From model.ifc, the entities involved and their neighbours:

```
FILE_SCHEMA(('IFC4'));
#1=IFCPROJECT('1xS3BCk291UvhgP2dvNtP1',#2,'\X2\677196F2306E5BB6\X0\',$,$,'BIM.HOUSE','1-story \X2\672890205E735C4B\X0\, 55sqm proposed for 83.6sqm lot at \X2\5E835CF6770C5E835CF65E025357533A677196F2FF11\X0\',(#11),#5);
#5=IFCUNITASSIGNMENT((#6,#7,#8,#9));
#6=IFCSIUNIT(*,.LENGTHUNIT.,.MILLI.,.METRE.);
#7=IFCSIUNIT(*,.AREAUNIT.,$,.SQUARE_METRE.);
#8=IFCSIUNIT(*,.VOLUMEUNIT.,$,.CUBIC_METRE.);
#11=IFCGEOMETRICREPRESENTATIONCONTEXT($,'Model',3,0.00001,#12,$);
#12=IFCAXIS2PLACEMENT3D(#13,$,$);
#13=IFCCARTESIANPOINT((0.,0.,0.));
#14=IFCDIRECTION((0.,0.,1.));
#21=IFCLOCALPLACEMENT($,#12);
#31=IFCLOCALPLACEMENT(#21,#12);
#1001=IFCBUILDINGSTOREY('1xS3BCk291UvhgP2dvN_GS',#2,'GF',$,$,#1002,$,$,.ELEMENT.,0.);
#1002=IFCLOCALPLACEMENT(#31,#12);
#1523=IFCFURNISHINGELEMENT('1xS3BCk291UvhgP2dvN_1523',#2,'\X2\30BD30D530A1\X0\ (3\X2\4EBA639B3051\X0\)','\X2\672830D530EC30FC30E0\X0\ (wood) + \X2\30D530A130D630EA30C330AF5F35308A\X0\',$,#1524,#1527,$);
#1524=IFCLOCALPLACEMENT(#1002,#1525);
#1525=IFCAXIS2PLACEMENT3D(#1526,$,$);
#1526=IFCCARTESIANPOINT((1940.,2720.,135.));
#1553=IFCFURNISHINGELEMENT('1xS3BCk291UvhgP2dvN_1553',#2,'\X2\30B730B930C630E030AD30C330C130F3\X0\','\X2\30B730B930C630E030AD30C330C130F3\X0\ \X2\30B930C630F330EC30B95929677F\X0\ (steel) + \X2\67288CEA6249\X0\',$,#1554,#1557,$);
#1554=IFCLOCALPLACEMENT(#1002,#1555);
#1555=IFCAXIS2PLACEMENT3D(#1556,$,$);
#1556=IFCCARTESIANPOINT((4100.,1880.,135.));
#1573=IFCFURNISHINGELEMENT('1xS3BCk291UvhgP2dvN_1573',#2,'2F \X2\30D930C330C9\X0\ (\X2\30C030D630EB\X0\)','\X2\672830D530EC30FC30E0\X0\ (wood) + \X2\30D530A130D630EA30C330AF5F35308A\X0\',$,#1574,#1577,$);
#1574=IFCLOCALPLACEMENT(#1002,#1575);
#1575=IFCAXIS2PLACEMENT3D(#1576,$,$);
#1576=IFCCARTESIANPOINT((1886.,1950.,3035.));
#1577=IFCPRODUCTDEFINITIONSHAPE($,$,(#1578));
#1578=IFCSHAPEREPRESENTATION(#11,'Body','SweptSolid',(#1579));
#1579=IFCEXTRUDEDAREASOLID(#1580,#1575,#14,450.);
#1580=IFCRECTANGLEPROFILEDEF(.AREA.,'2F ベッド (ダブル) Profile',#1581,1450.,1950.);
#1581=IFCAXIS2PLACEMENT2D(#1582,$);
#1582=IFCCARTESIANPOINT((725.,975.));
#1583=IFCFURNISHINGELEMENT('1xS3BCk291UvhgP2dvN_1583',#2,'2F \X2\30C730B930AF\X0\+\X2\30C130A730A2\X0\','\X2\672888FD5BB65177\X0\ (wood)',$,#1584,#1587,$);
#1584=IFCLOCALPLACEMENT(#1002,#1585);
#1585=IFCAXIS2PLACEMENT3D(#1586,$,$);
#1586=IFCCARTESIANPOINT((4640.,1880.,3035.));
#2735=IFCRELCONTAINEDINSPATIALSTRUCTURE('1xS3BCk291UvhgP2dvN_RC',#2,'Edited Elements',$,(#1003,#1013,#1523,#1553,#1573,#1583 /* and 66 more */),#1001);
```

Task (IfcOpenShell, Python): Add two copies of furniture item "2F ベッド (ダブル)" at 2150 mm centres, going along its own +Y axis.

```python
import ifcopenshell
import ifcopenshell.api.geometry
import ifcopenshell.api.root
import ifcopenshell.util.element
import ifcopenshell.util.placement
import ifcopenshell.util.unit

model = ifcopenshell.open("model.ifc")
unit_scale = ifcopenshell.util.unit.calculate_unit_scale(model)


def reuse_history(source, copy):
    """copy_class also copies each property set's owner history, people and application; keep the originals."""
    for rel in copy.IsDefinedBy:
        if rel.is_a("IfcRelDefinesByProperties") and (history := rel.RelatingPropertyDefinition.OwnerHistory):
            rel.RelatingPropertyDefinition.OwnerHistory = source.OwnerHistory
            ifcopenshell.util.element.remove_deep2(model, history)


source = model.by_guid("1xS3BCk291UvhgP2dvN_1573")
base = ifcopenshell.util.placement.get_local_placement(source.ObjectPlacement)
step = base[:3, 1] * 2.15 / unit_scale

for i in range(1, 3):
    copy = ifcopenshell.api.root.copy_class(model, product=source)
    copy.Representation = ifcopenshell.util.element.copy_deep(
        model, source.Representation, exclude=["IfcGeometricRepresentationContext", "IfcRepresentationMap"]
    )
    reuse_history(source, copy)
    matrix = base.copy()
    matrix[:3, 3] += i * step
    print("added at", matrix[:3, 3].round(3) + 0.0)
    ifcopenshell.api.geometry.edit_object_placement(model, product=copy, matrix=matrix, is_si=False)

model.write("model_edited.ifc")
```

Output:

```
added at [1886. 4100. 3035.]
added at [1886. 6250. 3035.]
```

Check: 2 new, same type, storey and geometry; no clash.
